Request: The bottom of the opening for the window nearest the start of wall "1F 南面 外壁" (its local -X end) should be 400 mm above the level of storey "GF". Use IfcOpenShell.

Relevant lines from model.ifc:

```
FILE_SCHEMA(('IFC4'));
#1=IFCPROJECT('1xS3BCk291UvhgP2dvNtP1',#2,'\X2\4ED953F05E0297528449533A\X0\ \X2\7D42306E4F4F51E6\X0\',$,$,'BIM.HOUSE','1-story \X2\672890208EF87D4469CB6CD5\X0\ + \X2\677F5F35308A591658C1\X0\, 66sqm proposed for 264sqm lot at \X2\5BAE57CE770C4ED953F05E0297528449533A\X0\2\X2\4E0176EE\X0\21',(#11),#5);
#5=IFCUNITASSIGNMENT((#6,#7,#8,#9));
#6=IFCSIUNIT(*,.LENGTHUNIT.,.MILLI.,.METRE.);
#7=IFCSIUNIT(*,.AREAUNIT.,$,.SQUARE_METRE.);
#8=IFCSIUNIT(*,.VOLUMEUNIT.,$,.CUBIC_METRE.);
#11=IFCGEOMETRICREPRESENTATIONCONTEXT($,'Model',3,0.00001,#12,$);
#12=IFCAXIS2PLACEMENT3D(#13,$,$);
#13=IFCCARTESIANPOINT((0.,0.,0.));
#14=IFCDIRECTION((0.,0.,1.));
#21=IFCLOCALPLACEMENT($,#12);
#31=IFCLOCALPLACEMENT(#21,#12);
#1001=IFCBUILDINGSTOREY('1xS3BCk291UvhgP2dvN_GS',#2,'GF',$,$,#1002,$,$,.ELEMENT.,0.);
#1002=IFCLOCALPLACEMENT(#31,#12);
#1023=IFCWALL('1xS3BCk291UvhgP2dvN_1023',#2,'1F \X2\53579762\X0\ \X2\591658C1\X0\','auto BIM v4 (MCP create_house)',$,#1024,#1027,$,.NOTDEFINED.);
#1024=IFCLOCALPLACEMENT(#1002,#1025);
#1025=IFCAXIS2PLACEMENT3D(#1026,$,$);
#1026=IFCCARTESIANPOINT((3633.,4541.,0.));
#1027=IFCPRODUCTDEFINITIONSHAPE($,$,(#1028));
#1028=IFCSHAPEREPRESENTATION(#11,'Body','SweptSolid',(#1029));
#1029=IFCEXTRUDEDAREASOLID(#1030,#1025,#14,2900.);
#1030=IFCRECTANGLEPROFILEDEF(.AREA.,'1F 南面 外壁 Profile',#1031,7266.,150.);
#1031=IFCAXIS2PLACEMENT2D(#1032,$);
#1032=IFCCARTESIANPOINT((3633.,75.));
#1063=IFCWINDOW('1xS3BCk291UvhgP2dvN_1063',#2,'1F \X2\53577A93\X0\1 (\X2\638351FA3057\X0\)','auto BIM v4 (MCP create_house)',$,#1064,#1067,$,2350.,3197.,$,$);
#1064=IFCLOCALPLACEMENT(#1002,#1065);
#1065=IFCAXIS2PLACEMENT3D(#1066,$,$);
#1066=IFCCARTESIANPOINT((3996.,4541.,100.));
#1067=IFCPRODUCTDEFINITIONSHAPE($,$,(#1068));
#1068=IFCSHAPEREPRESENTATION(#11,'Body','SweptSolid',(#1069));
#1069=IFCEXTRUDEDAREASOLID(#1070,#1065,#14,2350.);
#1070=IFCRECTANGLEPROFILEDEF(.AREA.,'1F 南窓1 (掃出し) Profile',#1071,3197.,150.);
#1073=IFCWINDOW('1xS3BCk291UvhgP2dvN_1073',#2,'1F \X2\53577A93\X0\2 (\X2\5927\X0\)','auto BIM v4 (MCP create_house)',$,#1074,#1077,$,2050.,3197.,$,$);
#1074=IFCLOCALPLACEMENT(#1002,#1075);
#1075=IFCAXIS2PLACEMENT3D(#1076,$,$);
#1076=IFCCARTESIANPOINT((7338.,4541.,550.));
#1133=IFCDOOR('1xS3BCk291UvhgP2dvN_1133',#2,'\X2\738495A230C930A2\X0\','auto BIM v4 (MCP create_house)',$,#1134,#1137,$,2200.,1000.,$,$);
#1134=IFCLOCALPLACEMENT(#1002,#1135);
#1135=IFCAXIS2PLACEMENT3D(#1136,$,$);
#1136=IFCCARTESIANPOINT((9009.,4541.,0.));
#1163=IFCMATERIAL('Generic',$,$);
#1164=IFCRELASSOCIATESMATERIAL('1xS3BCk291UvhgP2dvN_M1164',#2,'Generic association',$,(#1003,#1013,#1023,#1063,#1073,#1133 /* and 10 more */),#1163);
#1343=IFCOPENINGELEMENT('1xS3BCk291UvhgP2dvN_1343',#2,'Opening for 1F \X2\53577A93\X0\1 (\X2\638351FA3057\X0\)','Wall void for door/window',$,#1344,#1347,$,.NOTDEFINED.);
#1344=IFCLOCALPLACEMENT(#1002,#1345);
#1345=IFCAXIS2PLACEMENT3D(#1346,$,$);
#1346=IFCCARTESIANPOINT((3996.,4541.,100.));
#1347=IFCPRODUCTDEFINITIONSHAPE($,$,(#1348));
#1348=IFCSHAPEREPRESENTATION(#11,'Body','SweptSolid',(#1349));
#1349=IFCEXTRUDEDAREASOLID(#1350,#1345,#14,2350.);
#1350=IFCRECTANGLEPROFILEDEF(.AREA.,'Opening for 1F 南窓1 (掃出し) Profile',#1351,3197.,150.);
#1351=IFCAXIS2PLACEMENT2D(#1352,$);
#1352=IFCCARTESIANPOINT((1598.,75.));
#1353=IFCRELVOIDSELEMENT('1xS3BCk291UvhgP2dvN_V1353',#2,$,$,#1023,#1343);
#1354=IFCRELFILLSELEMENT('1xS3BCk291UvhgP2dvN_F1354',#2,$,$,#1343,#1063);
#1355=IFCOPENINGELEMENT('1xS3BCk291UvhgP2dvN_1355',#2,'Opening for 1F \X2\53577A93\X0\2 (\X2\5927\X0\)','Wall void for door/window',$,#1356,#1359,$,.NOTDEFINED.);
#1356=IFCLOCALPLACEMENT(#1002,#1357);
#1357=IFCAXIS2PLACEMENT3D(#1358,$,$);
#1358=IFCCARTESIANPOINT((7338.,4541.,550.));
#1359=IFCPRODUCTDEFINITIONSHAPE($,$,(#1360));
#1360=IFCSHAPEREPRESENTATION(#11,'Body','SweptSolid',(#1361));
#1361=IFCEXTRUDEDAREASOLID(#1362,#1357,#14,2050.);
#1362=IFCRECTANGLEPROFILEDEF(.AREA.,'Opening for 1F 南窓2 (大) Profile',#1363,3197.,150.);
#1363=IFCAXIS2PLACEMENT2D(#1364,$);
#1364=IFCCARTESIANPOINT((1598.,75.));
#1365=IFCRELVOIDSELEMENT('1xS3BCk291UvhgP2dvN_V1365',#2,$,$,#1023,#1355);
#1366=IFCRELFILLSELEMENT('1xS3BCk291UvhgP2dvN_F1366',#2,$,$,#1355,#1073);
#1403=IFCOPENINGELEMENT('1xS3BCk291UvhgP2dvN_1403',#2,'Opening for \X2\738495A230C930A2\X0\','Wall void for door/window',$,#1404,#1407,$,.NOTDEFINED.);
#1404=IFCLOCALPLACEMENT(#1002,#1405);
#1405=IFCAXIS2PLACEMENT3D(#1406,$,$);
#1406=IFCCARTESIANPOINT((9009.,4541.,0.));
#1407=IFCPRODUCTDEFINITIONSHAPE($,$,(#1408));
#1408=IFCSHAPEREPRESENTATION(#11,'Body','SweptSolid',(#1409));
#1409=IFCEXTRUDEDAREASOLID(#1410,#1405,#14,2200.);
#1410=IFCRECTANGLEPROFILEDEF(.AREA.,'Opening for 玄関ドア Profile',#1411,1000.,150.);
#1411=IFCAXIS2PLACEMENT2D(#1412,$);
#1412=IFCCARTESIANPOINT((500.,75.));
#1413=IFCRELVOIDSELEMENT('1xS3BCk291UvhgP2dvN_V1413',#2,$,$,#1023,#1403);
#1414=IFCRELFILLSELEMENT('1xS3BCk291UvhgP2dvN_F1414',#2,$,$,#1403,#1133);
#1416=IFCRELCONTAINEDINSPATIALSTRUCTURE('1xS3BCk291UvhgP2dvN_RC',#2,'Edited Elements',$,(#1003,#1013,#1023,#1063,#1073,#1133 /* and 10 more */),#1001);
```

```python
import numpy as np
import ifcopenshell
import ifcopenshell.api.geometry
import ifcopenshell.geom
import ifcopenshell.util.element
import ifcopenshell.util.placement
import ifcopenshell.util.shape
import ifcopenshell.util.unit

model = ifcopenshell.open("model.ifc")
unit_scale = ifcopenshell.util.unit.calculate_unit_scale(model)

window = model.by_guid("1xS3BCk291UvhgP2dvN_1063")
opening = window.FillsVoids[0].RelatingOpeningElement
storey = ifcopenshell.util.element.get_container(window, ifc_class="IfcBuildingStorey")
level = ifcopenshell.util.placement.get_local_placement(storey.ObjectPlacement)[2, 3]

# The opening's origin need not be at the sill, so measure its lowest point.
shape = ifcopenshell.geom.create_shape(ifcopenshell.geom.settings(), opening)
bottom = ifcopenshell.util.shape.get_shape_bottom_elevation(shape, shape.geometry) / unit_scale
dz = level + 0.4 / unit_scale - bottom

shift = np.array([0.0, 0.0, dz])
# The window is not placed relative to its opening, so move both.
for product in (opening, window):
    matrix = ifcopenshell.util.placement.get_local_placement(product.ObjectPlacement)
    matrix[:3, 3] += shift
    ifcopenshell.api.geometry.edit_object_placement(model, product=product, matrix=matrix, is_si=False)

print(f"moved by {dz * unit_scale:+.3f} m")

model.write("model_updated.ifc")
```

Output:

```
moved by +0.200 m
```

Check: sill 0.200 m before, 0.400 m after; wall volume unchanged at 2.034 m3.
